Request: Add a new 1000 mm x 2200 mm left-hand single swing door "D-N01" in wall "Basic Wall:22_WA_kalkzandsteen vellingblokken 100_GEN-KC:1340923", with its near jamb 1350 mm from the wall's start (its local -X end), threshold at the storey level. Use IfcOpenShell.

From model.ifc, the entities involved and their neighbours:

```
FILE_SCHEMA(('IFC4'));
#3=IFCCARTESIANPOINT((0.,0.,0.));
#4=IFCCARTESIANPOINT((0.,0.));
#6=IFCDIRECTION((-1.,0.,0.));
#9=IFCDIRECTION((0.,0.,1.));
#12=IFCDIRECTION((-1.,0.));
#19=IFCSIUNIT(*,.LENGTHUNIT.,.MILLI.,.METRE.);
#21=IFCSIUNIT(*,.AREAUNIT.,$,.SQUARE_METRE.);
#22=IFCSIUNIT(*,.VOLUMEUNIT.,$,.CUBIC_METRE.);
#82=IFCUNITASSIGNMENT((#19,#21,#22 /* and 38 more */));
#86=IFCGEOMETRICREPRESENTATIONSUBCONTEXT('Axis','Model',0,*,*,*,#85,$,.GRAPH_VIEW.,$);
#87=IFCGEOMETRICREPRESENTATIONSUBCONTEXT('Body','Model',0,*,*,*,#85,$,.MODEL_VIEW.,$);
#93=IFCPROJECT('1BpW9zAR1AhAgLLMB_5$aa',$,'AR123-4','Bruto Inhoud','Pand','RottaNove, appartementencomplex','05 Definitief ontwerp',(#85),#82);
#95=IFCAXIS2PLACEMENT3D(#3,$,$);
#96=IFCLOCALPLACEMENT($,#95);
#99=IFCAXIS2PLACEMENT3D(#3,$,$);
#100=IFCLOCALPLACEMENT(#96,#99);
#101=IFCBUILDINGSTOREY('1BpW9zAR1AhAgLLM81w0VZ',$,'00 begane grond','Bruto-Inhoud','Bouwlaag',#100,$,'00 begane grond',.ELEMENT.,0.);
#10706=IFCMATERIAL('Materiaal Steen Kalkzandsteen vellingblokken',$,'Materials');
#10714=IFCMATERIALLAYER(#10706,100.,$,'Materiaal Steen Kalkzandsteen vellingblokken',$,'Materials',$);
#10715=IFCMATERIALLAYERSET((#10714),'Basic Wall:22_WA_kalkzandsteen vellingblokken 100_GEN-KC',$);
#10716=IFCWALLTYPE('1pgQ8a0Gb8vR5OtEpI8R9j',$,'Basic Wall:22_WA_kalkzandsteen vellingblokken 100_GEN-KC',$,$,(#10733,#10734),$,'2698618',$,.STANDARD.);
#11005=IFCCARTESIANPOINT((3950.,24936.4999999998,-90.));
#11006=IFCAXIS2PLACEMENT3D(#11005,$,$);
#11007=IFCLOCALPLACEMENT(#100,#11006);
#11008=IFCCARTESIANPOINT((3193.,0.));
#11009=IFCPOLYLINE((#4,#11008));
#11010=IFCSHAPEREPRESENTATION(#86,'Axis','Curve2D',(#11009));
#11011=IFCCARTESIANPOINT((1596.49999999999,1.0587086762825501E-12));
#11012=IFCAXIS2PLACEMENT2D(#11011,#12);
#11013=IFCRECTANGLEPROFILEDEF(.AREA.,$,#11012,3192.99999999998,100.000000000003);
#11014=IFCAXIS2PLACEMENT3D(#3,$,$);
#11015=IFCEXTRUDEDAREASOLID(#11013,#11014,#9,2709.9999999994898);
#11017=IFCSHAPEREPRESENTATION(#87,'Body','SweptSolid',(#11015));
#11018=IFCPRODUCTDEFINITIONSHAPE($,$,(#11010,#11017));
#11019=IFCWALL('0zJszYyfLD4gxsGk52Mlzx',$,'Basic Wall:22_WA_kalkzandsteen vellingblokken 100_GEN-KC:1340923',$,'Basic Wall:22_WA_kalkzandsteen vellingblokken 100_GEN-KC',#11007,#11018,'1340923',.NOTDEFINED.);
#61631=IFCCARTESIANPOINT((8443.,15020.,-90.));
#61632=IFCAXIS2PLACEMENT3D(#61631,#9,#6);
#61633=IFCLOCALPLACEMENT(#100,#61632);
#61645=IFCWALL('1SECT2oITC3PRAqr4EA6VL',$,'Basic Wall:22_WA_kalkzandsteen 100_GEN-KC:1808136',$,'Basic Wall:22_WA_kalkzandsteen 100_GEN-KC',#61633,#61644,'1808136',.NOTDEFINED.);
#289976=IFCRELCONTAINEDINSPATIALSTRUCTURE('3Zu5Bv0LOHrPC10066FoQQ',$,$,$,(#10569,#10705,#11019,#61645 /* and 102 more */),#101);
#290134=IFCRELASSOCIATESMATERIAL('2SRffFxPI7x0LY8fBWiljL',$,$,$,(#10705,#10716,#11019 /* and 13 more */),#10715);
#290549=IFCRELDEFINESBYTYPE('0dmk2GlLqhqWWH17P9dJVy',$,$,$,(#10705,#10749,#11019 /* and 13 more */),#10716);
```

```python
import numpy as np
import ifcopenshell
import ifcopenshell.api.feature
import ifcopenshell.api.geometry
import ifcopenshell.api.root
import ifcopenshell.api.spatial
import ifcopenshell.geom
import ifcopenshell.util.element
import ifcopenshell.util.placement
import ifcopenshell.util.representation
import ifcopenshell.util.shape
import ifcopenshell.util.unit

model = ifcopenshell.open("model.ifc")
unit_scale = ifcopenshell.util.unit.calculate_unit_scale(model)
settings = ifcopenshell.geom.settings()


def volume(element):
    """Net volume in cubic metres, openings subtracted."""
    shape = ifcopenshell.geom.create_shape(settings, element)
    return ifcopenshell.util.shape.get_volume(shape.geometry)


wall = model.by_guid("0zJszYyfLD4gxsGk52Mlzx")
storey = ifcopenshell.util.element.get_container(wall, ifc_class="IfcBuildingStorey")
context = ifcopenshell.util.representation.get_context(model, "Model", "Body", "MODEL_VIEW")
before = volume(wall)

width, height, from_end, sill = 1, 2.2, 1.35, 0.0  # metres

# The wall runs along its own X axis, and the end named is its -X end.
wall_shape = ifcopenshell.geom.create_shape(settings, wall)
x, y, z = ifcopenshell.util.shape.get_vertices(wall_shape.geometry).T
start = x.min() + from_end
face, thickness = float(y.min()), float(y.max() - y.min())
wall_matrix = ifcopenshell.util.placement.get_local_placement(wall.ObjectPlacement)
level = ifcopenshell.util.placement.get_local_placement(storey.ObjectPlacement)[2, 3]


def in_wall(x, y):
    """Placement at x, y metres in the wall's axes, at sill height."""
    matrix = wall_matrix.copy()
    matrix[:, 3] = wall_matrix @ np.array([x / unit_scale, y / unit_scale, 0.0, 1.0])
    matrix[2, 3] = level + sill / unit_scale
    return matrix


# Opening: a box that overshoots both wall faces by 50 mm.
opening = ifcopenshell.api.root.create_entity(model, ifc_class="IfcOpeningElement", predefined_type="OPENING")
box = ifcopenshell.api.geometry.add_wall_representation(
    model, context=context, length=width, height=height, thickness=thickness + 0.1
)
ifcopenshell.api.geometry.assign_representation(model, product=opening, representation=box)
ifcopenshell.api.geometry.edit_object_placement(model, product=opening, matrix=in_wall(start, face - 0.05), is_si=False)
ifcopenshell.api.feature.add_feature(model, feature=opening, element=wall)

door = ifcopenshell.api.root.create_entity(model, ifc_class="IfcDoor", name="D-N01", predefined_type="DOOR")
door.OverallWidth, door.OverallHeight = width / unit_scale, height / unit_scale
door.OperationType = "SINGLE_SWING_LEFT"
body = ifcopenshell.api.geometry.add_door_representation(
    model,
    context=context,
    overall_width=door.OverallWidth,
    overall_height=door.OverallHeight,
    operation_type="SINGLE_SWING_LEFT",
    lining_properties={"LiningDepth": thickness / unit_scale, "ThresholdDepth": thickness / unit_scale},
)
ifcopenshell.api.geometry.assign_representation(model, product=door, representation=body)
ifcopenshell.api.spatial.assign_container(model, products=[door], relating_structure=storey)
ifcopenshell.api.feature.add_filling(model, opening=opening, element=door)

# The lining spans the wall, so the door starts at the wall face.
ifcopenshell.api.geometry.edit_object_placement(model, product=door, matrix=in_wall(start, face), is_si=False)

after = volume(wall)

print(f"wall volume {before:.3f} -> {after:.3f} m3")

model.write("model_v2.ifc")
```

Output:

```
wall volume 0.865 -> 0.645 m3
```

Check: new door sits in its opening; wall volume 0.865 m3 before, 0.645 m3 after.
